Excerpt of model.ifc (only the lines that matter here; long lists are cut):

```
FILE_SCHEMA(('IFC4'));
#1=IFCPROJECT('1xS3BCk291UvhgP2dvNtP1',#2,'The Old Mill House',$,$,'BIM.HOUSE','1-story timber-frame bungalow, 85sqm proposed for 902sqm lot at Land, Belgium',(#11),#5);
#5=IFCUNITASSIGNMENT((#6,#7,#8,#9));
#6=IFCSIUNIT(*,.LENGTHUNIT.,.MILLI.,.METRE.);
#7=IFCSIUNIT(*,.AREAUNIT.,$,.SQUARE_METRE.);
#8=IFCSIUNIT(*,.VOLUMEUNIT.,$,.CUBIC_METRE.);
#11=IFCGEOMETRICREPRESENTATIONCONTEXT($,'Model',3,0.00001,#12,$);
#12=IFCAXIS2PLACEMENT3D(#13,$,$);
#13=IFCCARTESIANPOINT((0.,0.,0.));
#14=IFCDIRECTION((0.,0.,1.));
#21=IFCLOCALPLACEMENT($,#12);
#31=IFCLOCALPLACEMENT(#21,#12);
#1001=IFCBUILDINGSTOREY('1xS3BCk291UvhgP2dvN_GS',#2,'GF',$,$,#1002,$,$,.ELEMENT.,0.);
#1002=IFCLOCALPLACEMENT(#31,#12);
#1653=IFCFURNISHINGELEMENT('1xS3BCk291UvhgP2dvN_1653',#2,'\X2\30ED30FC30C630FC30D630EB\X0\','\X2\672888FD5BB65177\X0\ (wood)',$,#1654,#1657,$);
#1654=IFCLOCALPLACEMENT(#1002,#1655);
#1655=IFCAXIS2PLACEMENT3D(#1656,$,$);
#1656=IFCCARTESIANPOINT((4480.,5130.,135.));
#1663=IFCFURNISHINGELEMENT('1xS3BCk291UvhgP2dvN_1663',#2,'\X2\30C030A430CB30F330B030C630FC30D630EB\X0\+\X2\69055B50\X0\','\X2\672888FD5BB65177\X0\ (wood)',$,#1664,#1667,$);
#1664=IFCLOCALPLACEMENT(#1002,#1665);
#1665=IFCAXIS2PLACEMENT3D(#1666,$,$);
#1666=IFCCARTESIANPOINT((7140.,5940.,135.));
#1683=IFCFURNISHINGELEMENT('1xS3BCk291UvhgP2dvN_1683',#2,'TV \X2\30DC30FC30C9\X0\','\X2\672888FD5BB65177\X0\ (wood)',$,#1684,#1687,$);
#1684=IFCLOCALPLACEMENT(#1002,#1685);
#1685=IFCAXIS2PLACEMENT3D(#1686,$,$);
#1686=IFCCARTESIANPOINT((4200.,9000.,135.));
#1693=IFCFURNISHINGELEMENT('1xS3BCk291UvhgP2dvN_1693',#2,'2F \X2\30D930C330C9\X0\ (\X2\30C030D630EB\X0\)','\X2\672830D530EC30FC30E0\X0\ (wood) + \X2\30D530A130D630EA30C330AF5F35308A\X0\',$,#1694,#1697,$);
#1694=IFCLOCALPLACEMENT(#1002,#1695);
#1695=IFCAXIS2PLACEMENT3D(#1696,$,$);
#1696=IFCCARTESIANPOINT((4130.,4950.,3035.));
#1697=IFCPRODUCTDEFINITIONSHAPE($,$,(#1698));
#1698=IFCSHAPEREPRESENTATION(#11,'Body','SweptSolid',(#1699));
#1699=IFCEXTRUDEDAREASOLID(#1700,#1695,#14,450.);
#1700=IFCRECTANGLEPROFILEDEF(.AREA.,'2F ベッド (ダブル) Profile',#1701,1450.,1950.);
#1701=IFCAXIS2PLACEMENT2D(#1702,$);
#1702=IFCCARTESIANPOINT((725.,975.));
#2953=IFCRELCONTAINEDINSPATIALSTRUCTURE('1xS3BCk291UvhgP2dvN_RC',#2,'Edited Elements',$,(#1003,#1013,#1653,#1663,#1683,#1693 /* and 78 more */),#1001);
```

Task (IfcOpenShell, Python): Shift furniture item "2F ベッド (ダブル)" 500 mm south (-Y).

```python
import ifcopenshell
import ifcopenshell.api.geometry
import ifcopenshell.util.placement

model = ifcopenshell.open("model.ifc")

item = model.by_guid("1xS3BCk291UvhgP2dvN_1693")
matrix = ifcopenshell.util.placement.get_local_placement(item.ObjectPlacement)
matrix[1, 3] -= 500.0
ifcopenshell.api.geometry.edit_object_placement(model, product=item, matrix=matrix, is_si=False)

print(ifcopenshell.util.placement.get_local_placement(item.ObjectPlacement).round(3) + 0.0)

model.write("model-out.ifc")
```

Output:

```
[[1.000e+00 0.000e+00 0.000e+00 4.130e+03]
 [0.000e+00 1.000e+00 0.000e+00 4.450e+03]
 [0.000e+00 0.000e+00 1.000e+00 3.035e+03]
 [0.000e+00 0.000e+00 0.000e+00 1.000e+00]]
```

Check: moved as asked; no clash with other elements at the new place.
